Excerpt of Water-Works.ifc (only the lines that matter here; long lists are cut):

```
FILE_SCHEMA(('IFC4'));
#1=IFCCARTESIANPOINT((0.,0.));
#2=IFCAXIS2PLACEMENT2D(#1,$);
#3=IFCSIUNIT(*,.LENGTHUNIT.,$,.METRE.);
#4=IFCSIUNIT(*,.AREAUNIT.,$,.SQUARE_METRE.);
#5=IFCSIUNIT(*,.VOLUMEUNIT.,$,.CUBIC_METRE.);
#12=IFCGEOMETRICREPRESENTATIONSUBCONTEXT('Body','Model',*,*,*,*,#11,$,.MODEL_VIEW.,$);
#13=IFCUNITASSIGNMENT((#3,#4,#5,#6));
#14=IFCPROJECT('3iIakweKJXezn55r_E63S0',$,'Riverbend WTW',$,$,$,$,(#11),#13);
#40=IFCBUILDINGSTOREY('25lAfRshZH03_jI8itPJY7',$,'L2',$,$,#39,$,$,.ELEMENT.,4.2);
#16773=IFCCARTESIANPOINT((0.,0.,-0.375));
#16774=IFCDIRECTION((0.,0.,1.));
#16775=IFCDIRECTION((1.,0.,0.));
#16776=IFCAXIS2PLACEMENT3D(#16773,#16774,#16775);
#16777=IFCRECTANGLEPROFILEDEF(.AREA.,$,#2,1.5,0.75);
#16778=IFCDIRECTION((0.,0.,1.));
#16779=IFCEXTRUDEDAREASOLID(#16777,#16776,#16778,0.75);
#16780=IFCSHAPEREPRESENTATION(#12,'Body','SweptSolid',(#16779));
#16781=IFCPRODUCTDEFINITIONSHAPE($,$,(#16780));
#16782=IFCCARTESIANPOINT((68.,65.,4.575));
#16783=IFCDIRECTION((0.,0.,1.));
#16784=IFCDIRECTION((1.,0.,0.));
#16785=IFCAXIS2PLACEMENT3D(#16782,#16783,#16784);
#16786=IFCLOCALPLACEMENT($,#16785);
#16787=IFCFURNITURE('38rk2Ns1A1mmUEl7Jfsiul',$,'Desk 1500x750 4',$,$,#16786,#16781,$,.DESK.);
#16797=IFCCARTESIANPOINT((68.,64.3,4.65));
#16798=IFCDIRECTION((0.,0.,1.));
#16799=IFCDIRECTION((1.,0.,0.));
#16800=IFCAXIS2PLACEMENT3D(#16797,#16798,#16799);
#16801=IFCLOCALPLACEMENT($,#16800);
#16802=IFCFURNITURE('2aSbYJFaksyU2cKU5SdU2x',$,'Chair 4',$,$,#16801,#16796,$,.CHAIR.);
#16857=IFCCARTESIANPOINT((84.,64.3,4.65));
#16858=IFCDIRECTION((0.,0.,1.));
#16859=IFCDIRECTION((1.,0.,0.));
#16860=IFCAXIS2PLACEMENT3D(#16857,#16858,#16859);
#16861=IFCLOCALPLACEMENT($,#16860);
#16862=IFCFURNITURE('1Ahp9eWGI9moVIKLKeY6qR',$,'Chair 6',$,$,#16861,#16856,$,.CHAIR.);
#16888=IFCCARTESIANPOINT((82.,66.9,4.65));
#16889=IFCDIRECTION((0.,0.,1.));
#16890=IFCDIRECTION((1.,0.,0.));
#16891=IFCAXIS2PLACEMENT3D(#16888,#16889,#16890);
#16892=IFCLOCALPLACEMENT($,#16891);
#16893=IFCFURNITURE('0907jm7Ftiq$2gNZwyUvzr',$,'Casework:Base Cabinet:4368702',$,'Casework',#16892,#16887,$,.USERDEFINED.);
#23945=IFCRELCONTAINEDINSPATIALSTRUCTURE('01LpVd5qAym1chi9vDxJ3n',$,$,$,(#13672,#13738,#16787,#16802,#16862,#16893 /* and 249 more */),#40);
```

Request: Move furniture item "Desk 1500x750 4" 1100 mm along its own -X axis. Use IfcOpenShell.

```python
import ifcopenshell
import ifcopenshell.api.geometry
import ifcopenshell.util.placement
import ifcopenshell.util.unit

model = ifcopenshell.open("Water-Works.ifc")
unit_scale = ifcopenshell.util.unit.calculate_unit_scale(model)

item = model.by_guid("38rk2Ns1A1mmUEl7Jfsiul")
matrix = ifcopenshell.util.placement.get_local_placement(item.ObjectPlacement)
matrix[:3, 3] -= matrix[:3, 0] * 1.1 / unit_scale
ifcopenshell.api.geometry.edit_object_placement(model, product=item, matrix=matrix, is_si=False)

print(ifcopenshell.util.placement.get_local_placement(item.ObjectPlacement).round(3) + 0.0)

model.write("Water-Works_updated.ifc")
```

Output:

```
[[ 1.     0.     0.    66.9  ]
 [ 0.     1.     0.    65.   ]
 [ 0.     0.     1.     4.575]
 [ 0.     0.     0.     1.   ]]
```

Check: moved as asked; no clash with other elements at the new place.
